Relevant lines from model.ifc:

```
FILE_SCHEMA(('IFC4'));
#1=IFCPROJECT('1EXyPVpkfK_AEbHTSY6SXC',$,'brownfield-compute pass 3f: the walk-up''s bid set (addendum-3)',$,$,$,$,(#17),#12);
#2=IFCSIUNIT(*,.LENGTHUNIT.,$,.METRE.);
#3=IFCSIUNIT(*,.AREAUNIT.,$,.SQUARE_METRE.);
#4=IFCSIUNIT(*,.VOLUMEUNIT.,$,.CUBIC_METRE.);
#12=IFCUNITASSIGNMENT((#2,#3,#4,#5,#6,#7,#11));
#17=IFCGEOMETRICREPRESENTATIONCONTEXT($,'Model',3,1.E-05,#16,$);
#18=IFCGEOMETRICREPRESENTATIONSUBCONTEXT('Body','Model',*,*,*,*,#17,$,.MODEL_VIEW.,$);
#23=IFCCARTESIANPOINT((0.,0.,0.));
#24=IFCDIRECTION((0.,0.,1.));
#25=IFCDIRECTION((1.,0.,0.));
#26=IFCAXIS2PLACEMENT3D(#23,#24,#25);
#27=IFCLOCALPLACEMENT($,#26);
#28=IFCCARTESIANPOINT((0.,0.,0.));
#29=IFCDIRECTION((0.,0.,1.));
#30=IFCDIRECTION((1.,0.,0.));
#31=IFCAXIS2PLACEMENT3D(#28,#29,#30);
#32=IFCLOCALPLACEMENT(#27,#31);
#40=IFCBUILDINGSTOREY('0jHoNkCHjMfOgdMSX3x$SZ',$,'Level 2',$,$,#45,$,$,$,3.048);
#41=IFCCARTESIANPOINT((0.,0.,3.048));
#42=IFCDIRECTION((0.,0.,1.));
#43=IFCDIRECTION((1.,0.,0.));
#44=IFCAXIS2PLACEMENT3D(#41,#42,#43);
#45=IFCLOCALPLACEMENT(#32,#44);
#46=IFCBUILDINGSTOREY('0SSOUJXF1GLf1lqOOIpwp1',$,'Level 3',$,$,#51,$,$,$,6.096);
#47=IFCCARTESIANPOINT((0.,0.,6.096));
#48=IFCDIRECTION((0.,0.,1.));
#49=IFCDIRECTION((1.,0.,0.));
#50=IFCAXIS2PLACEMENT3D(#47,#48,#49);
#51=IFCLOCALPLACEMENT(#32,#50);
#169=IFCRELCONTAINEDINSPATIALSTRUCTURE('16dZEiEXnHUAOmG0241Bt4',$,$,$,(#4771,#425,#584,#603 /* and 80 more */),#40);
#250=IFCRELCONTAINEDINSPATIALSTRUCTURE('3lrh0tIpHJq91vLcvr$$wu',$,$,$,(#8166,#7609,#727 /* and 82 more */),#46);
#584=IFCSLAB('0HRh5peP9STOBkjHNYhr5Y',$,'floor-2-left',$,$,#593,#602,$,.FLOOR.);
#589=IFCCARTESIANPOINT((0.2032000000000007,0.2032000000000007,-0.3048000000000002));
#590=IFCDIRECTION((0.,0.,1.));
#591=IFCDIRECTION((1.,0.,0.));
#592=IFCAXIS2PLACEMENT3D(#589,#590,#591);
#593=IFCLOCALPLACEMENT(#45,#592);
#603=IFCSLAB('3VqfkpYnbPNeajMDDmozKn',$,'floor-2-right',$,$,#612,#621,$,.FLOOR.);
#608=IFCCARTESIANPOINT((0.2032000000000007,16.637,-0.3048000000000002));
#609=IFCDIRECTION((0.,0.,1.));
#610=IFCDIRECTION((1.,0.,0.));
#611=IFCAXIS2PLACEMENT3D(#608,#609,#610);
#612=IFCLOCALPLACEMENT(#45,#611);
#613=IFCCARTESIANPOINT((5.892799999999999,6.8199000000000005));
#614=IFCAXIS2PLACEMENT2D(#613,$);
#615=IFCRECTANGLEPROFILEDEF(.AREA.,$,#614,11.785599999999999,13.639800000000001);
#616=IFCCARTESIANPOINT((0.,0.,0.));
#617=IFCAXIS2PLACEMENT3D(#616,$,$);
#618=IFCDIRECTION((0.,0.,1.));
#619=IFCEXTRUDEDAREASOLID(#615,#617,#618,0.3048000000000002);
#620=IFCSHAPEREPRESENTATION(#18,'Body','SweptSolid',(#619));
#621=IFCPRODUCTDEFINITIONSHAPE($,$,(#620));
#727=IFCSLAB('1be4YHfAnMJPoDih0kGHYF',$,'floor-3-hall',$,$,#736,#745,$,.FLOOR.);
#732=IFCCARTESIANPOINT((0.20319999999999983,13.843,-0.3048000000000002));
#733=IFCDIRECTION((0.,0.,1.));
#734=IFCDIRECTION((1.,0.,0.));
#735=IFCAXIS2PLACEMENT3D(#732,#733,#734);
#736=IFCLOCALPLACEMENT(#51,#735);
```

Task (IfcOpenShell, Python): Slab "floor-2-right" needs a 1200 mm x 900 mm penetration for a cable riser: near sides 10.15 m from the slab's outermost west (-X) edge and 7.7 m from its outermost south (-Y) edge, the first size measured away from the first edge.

```python
import numpy as np
import ifcopenshell
import ifcopenshell.api.feature
import ifcopenshell.api.geometry
import ifcopenshell.api.root
import ifcopenshell.geom
import ifcopenshell.util.placement
import ifcopenshell.util.representation
import ifcopenshell.util.shape
import ifcopenshell.util.unit

model = ifcopenshell.open("model.ifc")
unit_scale = ifcopenshell.util.unit.calculate_unit_scale(model)
settings = ifcopenshell.geom.settings()


def volume(element):
    """Net volume in cubic metres, openings subtracted."""
    shape = ifcopenshell.geom.create_shape(settings, element)
    return ifcopenshell.util.shape.get_volume(shape.geometry)


slab = model.by_guid("3VqfkpYnbPNeajMDDmozKn")
before = volume(slab)

# Extent in the slab's own axes, in metres. The edges named are its -X and -Y sides.
slab_shape = ifcopenshell.geom.create_shape(settings, slab)
vertices = ifcopenshell.util.shape.get_vertices(slab_shape.geometry)
x_min, y_min, bottom = vertices.min(axis=0)
top = vertices[:, 2].max()

opening = ifcopenshell.api.root.create_entity(model, ifc_class="IfcOpeningElement", name="Cable riser opening", predefined_type="OPENING")
context = ifcopenshell.util.representation.get_context(model, "Model", "Body", "MODEL_VIEW")
width, depth = 1.2, 0.9
outline = [(0.0, 0.0), (width, 0.0), (width, depth), (0.0, depth), (0.0, 0.0)]
# Overshoot both faces by 50 mm so the cut is clean.
shape = ifcopenshell.api.geometry.add_slab_representation(
    model, context=context, depth=top - bottom + 0.1, polyline=outline
)
ifcopenshell.api.geometry.assign_representation(model, product=opening, representation=shape)

matrix = ifcopenshell.util.placement.get_local_placement(slab.ObjectPlacement)
matrix[:, 3] = matrix @ np.append(np.array([x_min + 10.15, y_min + 7.7, bottom - 0.05]) / unit_scale, 1.0)
ifcopenshell.api.geometry.edit_object_placement(model, product=opening, matrix=matrix, is_si=False)
ifcopenshell.api.feature.add_feature(model, feature=opening, element=slab)

after = volume(slab)

print(f"slab volume {before:.3f} -> {after:.3f} m3")

model.write("model_v2.ifc")
```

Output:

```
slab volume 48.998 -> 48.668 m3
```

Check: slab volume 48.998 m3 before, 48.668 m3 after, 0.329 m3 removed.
